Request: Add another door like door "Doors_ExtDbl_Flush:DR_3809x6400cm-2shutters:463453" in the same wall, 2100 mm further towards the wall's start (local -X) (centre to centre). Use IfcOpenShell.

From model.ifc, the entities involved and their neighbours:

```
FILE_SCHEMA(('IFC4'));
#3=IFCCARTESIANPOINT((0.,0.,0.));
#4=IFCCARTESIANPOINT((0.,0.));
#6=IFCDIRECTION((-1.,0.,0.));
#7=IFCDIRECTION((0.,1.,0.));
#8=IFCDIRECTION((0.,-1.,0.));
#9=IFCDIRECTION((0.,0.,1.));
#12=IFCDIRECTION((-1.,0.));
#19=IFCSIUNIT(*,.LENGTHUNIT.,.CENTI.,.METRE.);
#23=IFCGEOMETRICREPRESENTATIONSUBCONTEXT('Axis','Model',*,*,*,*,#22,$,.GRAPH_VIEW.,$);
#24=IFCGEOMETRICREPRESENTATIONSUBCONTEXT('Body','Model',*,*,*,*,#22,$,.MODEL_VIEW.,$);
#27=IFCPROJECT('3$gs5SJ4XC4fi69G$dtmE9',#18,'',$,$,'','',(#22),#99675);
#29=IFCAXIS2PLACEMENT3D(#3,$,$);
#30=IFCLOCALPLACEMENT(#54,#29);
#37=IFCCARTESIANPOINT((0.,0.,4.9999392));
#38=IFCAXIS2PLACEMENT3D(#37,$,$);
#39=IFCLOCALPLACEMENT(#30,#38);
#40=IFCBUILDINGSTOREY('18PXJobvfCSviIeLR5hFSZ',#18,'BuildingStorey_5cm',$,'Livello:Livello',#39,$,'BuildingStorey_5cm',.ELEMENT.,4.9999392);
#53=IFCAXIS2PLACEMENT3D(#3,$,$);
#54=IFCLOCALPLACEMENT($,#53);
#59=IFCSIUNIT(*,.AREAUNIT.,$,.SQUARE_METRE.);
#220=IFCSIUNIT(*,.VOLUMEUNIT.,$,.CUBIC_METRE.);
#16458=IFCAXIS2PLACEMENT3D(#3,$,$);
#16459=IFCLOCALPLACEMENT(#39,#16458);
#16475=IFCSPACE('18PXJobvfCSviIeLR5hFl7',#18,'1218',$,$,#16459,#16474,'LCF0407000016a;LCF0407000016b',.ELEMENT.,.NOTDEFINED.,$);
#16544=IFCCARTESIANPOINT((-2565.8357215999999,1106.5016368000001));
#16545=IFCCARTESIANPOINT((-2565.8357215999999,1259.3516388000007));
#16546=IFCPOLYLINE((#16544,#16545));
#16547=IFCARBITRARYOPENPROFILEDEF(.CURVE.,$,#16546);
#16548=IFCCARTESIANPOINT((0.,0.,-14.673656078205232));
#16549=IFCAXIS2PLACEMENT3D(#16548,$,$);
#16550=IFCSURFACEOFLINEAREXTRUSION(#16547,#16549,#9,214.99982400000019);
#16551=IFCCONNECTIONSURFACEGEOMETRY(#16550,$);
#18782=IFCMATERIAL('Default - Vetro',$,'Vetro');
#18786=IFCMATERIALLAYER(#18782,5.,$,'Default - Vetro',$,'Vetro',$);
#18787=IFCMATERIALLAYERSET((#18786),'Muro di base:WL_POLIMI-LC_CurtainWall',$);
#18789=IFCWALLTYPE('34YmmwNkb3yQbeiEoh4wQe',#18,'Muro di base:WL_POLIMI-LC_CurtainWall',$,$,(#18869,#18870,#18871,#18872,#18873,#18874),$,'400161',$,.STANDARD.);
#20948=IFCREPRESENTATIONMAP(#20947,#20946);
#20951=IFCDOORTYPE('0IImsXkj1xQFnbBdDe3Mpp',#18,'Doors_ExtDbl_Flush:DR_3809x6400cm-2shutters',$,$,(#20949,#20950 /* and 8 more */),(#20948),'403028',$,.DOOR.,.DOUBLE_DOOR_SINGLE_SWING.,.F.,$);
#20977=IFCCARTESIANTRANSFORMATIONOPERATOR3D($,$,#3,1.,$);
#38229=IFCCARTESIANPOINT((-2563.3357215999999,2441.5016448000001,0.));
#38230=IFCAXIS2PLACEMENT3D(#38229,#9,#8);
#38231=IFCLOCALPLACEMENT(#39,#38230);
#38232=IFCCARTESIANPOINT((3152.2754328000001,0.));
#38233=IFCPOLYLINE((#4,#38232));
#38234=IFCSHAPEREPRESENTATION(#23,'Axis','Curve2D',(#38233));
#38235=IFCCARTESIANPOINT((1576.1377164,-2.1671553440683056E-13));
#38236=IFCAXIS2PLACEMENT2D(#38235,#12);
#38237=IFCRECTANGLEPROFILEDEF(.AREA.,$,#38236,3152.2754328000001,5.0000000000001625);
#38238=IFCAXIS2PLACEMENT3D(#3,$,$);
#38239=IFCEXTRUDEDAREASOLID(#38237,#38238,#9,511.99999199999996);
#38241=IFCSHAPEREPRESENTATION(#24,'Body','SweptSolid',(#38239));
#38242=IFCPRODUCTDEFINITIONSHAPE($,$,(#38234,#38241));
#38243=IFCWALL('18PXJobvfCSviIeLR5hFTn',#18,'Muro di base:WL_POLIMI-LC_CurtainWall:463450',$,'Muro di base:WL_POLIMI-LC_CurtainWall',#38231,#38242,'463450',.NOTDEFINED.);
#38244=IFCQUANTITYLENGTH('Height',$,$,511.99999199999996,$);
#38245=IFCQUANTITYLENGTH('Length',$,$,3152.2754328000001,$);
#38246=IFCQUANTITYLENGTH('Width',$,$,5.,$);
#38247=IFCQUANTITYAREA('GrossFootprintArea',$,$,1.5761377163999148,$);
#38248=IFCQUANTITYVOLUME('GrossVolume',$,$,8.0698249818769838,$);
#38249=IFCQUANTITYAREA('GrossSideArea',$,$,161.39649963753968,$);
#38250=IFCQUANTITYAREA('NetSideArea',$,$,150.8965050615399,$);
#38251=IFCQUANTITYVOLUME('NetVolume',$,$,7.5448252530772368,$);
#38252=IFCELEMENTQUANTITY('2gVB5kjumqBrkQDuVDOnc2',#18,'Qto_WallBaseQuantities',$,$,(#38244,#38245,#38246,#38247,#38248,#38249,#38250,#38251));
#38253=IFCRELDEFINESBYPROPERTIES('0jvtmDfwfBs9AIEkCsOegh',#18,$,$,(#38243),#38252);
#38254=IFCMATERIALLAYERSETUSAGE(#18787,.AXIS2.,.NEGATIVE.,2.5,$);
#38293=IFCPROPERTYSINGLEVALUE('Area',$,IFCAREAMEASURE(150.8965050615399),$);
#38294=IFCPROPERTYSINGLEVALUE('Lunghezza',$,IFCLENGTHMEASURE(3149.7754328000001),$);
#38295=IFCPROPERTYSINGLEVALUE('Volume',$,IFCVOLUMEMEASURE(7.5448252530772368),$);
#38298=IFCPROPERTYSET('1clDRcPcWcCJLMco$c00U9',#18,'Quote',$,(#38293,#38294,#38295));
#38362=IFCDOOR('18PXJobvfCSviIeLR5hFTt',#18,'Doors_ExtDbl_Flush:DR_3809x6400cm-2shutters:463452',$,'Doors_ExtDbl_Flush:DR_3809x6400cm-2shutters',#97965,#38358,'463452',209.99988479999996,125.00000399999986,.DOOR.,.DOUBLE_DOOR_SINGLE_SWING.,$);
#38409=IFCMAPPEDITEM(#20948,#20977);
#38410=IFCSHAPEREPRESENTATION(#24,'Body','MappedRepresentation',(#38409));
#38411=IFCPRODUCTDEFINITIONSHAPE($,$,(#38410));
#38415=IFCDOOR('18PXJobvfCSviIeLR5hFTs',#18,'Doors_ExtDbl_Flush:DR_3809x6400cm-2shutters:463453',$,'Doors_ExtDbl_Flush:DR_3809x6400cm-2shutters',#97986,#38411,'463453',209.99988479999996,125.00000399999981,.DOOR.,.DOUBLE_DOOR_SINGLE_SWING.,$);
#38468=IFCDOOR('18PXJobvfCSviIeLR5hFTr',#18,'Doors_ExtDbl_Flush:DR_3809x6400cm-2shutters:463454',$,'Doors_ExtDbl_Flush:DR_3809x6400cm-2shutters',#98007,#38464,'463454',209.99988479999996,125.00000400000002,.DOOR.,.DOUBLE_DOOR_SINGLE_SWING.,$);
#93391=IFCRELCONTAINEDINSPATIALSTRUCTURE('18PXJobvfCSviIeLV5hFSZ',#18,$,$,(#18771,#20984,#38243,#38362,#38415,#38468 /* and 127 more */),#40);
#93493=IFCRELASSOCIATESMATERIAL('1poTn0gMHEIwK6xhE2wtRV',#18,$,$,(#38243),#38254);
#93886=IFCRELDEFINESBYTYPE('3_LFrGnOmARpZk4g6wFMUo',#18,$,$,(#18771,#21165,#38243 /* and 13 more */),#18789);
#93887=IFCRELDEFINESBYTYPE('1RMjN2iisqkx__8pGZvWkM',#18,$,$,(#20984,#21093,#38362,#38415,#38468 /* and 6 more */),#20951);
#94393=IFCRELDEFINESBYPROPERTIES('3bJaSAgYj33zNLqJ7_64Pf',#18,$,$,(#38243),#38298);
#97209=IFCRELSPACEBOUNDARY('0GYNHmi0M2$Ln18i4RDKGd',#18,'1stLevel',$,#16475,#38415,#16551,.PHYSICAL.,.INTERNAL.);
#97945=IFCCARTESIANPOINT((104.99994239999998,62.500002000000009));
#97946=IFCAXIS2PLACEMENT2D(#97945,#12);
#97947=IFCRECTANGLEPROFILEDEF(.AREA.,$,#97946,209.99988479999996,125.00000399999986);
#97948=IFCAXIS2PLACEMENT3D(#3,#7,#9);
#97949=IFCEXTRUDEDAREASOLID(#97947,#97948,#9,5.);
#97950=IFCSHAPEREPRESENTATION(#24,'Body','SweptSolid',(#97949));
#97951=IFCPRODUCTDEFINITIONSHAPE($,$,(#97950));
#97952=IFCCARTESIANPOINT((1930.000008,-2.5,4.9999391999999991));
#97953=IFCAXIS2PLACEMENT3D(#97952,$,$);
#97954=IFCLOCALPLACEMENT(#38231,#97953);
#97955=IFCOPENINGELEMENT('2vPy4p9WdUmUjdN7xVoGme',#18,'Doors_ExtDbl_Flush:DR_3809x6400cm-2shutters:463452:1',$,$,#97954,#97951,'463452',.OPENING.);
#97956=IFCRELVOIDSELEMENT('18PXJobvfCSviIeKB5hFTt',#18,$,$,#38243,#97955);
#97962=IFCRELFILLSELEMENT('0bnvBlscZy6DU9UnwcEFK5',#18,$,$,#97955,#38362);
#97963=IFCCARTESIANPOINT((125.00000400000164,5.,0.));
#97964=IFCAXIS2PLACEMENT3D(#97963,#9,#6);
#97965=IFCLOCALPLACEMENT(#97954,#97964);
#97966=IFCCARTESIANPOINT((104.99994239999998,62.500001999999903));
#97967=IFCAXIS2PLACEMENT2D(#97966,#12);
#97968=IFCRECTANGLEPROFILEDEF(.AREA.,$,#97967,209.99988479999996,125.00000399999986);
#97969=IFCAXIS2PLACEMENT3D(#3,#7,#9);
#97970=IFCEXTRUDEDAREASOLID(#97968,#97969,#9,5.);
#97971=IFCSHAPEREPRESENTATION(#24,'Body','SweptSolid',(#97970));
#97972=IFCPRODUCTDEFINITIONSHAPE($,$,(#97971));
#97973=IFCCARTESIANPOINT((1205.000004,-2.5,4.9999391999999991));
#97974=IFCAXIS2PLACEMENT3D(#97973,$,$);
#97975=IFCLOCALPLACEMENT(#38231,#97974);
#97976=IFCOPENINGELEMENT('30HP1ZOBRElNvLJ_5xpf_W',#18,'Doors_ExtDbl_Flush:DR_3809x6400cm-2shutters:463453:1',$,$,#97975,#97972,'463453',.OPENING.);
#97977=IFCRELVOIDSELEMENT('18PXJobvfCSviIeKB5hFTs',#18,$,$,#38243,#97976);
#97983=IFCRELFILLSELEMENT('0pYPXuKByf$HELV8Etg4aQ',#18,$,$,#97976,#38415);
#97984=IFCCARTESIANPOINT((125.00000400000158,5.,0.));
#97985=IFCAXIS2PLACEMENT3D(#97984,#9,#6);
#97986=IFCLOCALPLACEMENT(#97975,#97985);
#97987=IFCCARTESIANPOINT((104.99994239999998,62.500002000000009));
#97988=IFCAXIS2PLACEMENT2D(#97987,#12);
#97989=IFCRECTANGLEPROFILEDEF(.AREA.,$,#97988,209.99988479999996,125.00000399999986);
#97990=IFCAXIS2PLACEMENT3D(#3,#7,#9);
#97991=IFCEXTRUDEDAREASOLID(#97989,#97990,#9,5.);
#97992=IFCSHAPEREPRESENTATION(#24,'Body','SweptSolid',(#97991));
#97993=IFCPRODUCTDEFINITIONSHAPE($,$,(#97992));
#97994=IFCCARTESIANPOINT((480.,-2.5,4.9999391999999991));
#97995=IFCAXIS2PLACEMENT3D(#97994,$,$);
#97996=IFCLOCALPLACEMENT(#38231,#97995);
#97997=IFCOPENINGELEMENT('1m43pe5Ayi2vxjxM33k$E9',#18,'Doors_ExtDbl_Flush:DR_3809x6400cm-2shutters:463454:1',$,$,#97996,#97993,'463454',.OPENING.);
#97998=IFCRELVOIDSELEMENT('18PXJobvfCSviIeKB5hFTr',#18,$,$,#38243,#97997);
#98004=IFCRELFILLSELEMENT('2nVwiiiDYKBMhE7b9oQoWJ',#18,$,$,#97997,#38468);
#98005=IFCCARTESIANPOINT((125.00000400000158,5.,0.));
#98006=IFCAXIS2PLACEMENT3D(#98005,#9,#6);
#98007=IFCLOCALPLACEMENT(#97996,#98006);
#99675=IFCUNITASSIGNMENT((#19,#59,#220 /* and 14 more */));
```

```python
import numpy as np
import ifcopenshell
import ifcopenshell.api.feature
import ifcopenshell.api.geometry
import ifcopenshell.api.pset
import ifcopenshell.api.root
import ifcopenshell.geom
import ifcopenshell.util.element
import ifcopenshell.util.placement
import ifcopenshell.util.shape
import ifcopenshell.util.unit

model = ifcopenshell.open("model.ifc")
unit_scale = ifcopenshell.util.unit.calculate_unit_scale(model)
area_scale = ifcopenshell.util.unit.calculate_unit_scale(model, "AREAUNIT")
volume_scale = ifcopenshell.util.unit.calculate_unit_scale(model, "VOLUMEUNIT")
settings = ifcopenshell.geom.settings()


def volume(element):
    """Net volume in cubic metres, openings subtracted."""
    shape = ifcopenshell.geom.create_shape(settings, element)
    return ifcopenshell.util.shape.get_volume(shape.geometry)


def reuse_history(source, copy):
    """copy_class also copies each property set's owner history, people and application; keep the originals."""
    for rel in copy.IsDefinedBy:
        if rel.is_a("IfcRelDefinesByProperties") and (history := rel.RelatingPropertyDefinition.OwnerHistory):
            rel.RelatingPropertyDefinition.OwnerHistory = source.OwnerHistory
            ifcopenshell.util.element.remove_deep2(model, history)


door = model.by_id(38415)
opening = door.FillsVoids[0].RelatingOpeningElement
wall = opening.VoidsElements[0].RelatingBuildingElement
before = volume(wall)
shift = ifcopenshell.util.placement.get_local_placement(wall.ObjectPlacement)[:3, 0] * -2.1 / unit_scale

# copy_class copies the void relationship, type, container and properties, but no geometry.
new_opening = ifcopenshell.api.root.copy_class(model, product=opening)
new_opening.Representation = ifcopenshell.util.element.copy_deep(
    model, opening.Representation, exclude=["IfcGeometricRepresentationContext", "IfcRepresentationMap"]
)
new_opening.Name = "Doors_ExtDbl_Flush:DR_3809x6400cm-2shutters"
new_opening.Tag = None
reuse_history(opening, new_opening)
new_door = ifcopenshell.api.root.copy_class(model, product=door)
new_door.Representation = ifcopenshell.util.element.copy_deep(
    model, door.Representation, exclude=["IfcGeometricRepresentationContext", "IfcRepresentationMap"]
)
new_door.Name = "Doors_ExtDbl_Flush:DR_3809x6400cm-2shutters"
new_door.Tag = None
reuse_history(door, new_door)
ifcopenshell.api.feature.add_filling(model, opening=new_opening, element=new_door)

for old, new in ((opening, new_opening), (door, new_door)):
    matrix = ifcopenshell.util.placement.get_local_placement(old.ObjectPlacement)
    matrix[:3, 3] += shift
    ifcopenshell.api.geometry.edit_object_placement(model, product=new, matrix=matrix, is_si=False)

# The copied space boundaries still share their surfaces with the original.
for rel in new_door.ProvidesBoundaries:
    if rel.ConnectionGeometry:
        rel.ConnectionGeometry = ifcopenshell.util.element.copy_deep(model, rel.ConnectionGeometry)

# Space boundary surfaces are stored in each space's coordinates; move them too.
for rel in new_door.ProvidesBoundaries:
    if not rel.ConnectionGeometry:
        continue
    surface = rel.ConnectionGeometry.SurfaceOnRelatingElement
    space_matrix = ifcopenshell.util.placement.get_local_placement(rel.RelatingSpace.ObjectPlacement)
    point = np.array(surface.Position.Location.Coordinates) + space_matrix[:3, :3].T @ shift
    surface.Position = model.createIfcAxis2Placement3D(
        model.createIfcCartesianPoint(point.tolist()), surface.Position.Axis, surface.Position.RefDirection
    )

after = volume(wall)
thickness = 0.05  # wall thickness in metres

# Update the wall's stored quantities.
qto = model.by_id(ifcopenshell.util.element.get_pset(wall, "Qto_WallBaseQuantities", should_inherit=False)["id"])
ifcopenshell.api.pset.edit_qto(model, qto=qto, properties={
    "NetSideArea": after / thickness / area_scale,
    "NetVolume": after / volume_scale,
})
pset = model.by_id(ifcopenshell.util.element.get_pset(wall, "Quote", should_inherit=False)["id"])
ifcopenshell.api.pset.edit_pset(model, pset=pset, properties={
    "Area": model.create_entity("IfcAreaMeasure", after / thickness / area_scale),
    "Volume": model.create_entity("IfcVolumeMeasure", after / volume_scale),
})

print(f"wall volume {before:.3f} -> {after:.3f} m3")

model.write("model_rev.ifc")
```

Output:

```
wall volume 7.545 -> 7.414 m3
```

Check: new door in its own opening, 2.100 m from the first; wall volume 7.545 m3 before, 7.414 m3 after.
